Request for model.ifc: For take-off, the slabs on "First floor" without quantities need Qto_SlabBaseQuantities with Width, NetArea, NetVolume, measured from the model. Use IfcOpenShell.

First a look at what the model holds.

```python
import ifcopenshell
import ifcopenshell.util.element
import ifcopenshell.util.unit

model = ifcopenshell.open("model.ifc")
print(model.schema)
for unit_type in ("LENGTHUNIT", "AREAUNIT", "VOLUMEUNIT"):
    print(unit_type, ifcopenshell.util.unit.calculate_unit_scale(model, unit_type))
storey = next(s for s in model.by_type("IfcBuildingStorey") if s.Name == "First floor")
slabs = [e for e in ifcopenshell.util.element.get_decomposition(storey) if e.is_a("IfcSlab")]
for e in sorted(slabs, key=lambda e: e.id()):
    print(e.id(), e.is_a(), e.Name, list(ifcopenshell.util.element.get_psets(e, qtos_only=True)), sep=" | ")
```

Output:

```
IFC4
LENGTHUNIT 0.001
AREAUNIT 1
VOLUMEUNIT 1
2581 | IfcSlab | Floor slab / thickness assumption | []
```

```python
import ifcopenshell
import ifcopenshell.api.pset
import ifcopenshell.geom
import ifcopenshell.util.element
import ifcopenshell.util.shape
import ifcopenshell.util.unit

model = ifcopenshell.open("model.ifc")
unit_scale = ifcopenshell.util.unit.calculate_unit_scale(model)
area_scale = ifcopenshell.util.unit.calculate_unit_scale(model, "AREAUNIT")
volume_scale = ifcopenshell.util.unit.calculate_unit_scale(model, "VOLUMEUNIT")
settings = ifcopenshell.geom.settings()

storey = next(s for s in model.by_type("IfcBuildingStorey") if s.Name == "First floor")
slabs = [e for e in ifcopenshell.util.element.get_decomposition(storey) if e.is_a("IfcSlab")]

for e in sorted(slabs, key=lambda e: e.id()):
    if ifcopenshell.util.element.get_psets(e, qtos_only=True, should_inherit=False):
        continue
    # Geometry comes back in metres, in the element's own axes.
    shape = ifcopenshell.geom.create_shape(settings, e)
    values = {
        "Width": ifcopenshell.util.shape.get_z(shape.geometry) / unit_scale,
        "NetArea": ifcopenshell.util.shape.get_footprint_area(shape.geometry) / area_scale,
        "NetVolume": ifcopenshell.util.shape.get_volume(shape.geometry) / volume_scale,
    }
    qto = ifcopenshell.api.pset.add_qto(model, product=e, name="Qto_SlabBaseQuantities")
    ifcopenshell.api.pset.edit_qto(model, qto=qto, properties=values)
    print(e.id(), {k: round(v, 3) for k, v in values.items()})

model.write("model-out.ifc")
```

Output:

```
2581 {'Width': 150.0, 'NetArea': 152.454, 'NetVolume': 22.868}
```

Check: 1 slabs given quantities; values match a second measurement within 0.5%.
